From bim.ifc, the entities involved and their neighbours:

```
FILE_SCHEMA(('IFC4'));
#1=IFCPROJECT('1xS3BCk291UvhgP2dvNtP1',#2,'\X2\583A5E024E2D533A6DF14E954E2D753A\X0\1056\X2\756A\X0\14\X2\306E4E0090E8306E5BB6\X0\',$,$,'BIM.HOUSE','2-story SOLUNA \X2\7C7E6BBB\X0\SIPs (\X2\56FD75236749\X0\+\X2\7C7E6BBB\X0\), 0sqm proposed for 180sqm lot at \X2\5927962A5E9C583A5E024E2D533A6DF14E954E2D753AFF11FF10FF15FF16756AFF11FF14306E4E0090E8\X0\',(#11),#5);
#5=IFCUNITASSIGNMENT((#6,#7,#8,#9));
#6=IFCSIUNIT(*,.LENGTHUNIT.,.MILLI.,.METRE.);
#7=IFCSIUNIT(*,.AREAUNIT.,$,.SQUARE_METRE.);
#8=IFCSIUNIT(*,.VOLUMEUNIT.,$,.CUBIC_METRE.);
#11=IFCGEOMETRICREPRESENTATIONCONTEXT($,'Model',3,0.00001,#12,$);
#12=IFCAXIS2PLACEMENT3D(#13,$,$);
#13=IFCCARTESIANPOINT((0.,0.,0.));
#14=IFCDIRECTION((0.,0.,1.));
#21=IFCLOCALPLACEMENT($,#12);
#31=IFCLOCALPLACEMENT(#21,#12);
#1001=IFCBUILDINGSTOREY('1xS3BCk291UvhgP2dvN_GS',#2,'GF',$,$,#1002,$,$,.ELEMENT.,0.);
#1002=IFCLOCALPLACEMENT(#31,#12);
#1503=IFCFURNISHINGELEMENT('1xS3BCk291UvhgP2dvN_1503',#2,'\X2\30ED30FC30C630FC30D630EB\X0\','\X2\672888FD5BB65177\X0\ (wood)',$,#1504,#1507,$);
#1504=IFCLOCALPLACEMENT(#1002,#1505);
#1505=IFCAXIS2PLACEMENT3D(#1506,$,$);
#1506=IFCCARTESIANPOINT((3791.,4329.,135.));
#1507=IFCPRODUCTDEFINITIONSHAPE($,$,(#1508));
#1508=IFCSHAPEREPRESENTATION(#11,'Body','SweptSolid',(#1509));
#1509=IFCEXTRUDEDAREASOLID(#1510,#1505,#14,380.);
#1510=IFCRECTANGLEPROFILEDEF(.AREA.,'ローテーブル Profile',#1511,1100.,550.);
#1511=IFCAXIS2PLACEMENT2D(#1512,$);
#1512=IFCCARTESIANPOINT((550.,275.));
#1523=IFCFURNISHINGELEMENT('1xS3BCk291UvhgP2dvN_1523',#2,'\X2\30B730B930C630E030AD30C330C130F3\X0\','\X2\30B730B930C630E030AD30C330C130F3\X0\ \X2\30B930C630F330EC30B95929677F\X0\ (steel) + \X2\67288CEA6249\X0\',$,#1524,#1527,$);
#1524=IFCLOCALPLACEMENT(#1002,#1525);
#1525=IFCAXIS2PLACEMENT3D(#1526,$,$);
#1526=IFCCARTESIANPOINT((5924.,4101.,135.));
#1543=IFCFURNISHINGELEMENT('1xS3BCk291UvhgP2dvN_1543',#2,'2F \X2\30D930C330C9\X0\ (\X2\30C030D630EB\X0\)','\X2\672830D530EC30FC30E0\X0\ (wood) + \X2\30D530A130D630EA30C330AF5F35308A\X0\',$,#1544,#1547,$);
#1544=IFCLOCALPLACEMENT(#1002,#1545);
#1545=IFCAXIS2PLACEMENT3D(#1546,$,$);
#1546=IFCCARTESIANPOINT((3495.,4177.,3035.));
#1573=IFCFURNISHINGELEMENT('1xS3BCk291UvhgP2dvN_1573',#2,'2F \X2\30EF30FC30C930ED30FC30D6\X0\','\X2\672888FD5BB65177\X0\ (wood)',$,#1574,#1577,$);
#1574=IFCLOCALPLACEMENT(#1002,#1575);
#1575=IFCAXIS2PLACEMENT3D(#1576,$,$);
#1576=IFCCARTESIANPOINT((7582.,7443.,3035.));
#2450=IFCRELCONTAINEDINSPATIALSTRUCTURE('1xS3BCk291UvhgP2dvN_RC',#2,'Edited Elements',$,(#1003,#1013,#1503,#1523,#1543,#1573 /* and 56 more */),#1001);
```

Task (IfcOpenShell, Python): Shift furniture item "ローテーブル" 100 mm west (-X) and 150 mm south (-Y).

```python
import ifcopenshell
import ifcopenshell.api.geometry
import ifcopenshell.util.placement

model = ifcopenshell.open("bim.ifc")

item = model.by_guid("1xS3BCk291UvhgP2dvN_1503")
matrix = ifcopenshell.util.placement.get_local_placement(item.ObjectPlacement)
matrix[0, 3] -= 100.0
matrix[1, 3] -= 150.0
ifcopenshell.api.geometry.edit_object_placement(model, product=item, matrix=matrix, is_si=False)

print(ifcopenshell.util.placement.get_local_placement(item.ObjectPlacement).round(3) + 0.0)

model.write("bim_updated.ifc")
```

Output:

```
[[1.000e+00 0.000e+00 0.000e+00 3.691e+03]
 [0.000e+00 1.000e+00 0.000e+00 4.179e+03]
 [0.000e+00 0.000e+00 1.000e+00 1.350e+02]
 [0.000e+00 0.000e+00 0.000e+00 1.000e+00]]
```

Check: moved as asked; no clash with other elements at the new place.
